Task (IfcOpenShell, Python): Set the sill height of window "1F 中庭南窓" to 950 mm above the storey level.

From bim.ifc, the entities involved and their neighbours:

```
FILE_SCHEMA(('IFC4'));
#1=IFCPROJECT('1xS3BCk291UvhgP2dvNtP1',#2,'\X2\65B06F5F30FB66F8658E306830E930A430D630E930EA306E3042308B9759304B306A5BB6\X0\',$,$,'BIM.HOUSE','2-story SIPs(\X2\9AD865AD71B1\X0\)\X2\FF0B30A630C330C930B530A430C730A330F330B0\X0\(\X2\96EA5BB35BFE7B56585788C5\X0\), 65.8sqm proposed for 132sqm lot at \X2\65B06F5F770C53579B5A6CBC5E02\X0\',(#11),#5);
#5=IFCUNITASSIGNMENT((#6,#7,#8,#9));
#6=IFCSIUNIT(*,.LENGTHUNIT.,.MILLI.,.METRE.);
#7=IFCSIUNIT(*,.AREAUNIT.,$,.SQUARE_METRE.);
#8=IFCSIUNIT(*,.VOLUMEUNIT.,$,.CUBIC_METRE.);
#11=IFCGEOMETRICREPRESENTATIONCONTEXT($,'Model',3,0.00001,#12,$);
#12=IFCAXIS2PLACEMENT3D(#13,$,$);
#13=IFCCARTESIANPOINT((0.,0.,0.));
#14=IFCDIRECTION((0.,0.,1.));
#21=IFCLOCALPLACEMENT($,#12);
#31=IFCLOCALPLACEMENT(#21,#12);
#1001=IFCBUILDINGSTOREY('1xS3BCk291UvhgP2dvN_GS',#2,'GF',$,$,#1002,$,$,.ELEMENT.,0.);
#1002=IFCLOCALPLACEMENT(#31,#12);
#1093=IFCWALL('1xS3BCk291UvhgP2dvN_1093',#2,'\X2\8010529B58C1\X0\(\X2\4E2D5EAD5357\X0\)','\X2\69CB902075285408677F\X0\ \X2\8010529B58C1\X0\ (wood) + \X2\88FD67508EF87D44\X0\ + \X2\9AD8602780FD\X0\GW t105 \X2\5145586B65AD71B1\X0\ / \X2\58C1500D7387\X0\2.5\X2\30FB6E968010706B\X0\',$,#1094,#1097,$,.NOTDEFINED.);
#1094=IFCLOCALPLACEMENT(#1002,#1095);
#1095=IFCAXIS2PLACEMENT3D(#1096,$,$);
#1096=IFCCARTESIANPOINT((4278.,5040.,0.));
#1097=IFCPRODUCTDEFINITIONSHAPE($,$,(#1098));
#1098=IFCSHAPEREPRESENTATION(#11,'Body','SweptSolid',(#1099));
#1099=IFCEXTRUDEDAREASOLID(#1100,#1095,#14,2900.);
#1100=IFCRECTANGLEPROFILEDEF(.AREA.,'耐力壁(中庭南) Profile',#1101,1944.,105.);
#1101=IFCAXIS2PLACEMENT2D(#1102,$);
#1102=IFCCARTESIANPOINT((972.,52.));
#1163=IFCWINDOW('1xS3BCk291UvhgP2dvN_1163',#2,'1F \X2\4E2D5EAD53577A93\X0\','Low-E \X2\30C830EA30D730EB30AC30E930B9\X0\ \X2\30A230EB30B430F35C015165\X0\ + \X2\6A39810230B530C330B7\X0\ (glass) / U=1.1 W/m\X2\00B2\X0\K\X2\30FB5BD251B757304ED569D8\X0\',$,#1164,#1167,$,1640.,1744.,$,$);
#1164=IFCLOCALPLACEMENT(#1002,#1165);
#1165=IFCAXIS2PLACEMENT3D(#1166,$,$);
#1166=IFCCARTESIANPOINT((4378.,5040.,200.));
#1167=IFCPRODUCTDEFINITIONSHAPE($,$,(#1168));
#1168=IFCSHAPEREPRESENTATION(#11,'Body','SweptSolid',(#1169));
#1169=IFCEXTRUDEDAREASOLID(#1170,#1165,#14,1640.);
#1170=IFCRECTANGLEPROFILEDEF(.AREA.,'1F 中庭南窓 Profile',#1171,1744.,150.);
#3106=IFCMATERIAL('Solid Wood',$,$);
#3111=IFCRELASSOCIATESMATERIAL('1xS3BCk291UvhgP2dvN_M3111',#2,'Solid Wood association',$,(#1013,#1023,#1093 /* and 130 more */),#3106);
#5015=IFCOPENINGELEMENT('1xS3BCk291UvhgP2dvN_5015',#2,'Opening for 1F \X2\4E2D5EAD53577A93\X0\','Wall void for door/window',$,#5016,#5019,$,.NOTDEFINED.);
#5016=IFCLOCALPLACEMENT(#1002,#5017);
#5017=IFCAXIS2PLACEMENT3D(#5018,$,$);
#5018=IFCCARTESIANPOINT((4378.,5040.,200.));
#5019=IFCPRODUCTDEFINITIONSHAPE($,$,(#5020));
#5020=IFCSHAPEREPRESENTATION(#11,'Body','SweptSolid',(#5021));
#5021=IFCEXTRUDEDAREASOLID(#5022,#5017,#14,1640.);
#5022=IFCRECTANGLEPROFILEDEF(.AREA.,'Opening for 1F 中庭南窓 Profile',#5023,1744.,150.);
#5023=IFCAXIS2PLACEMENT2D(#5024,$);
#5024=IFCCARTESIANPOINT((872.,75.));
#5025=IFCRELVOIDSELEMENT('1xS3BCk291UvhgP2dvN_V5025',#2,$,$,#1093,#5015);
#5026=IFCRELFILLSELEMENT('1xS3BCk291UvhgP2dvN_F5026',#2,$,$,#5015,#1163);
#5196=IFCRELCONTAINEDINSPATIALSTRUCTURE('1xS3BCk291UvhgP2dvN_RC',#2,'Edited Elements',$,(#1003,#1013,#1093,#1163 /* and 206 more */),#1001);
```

```python
import numpy as np
import ifcopenshell
import ifcopenshell.api.geometry
import ifcopenshell.geom
import ifcopenshell.util.element
import ifcopenshell.util.placement
import ifcopenshell.util.shape
import ifcopenshell.util.unit

model = ifcopenshell.open("bim.ifc")
unit_scale = ifcopenshell.util.unit.calculate_unit_scale(model)

window = model.by_guid("1xS3BCk291UvhgP2dvN_1163")
opening = window.FillsVoids[0].RelatingOpeningElement
storey = ifcopenshell.util.element.get_container(window, ifc_class="IfcBuildingStorey")
level = ifcopenshell.util.placement.get_local_placement(storey.ObjectPlacement)[2, 3]

# The opening's origin need not be at the sill, so measure its lowest point.
shape = ifcopenshell.geom.create_shape(ifcopenshell.geom.settings(), opening)
bottom = ifcopenshell.util.shape.get_shape_bottom_elevation(shape, shape.geometry) / unit_scale
dz = level + 950.0 - bottom

shift = np.array([0.0, 0.0, dz])
# The window is not placed relative to its opening, so move both.
for product in (opening, window):
    matrix = ifcopenshell.util.placement.get_local_placement(product.ObjectPlacement)
    matrix[:3, 3] += shift
    ifcopenshell.api.geometry.edit_object_placement(model, product=product, matrix=matrix, is_si=False)

print(f"moved by {dz * unit_scale:+.3f} m")

model.write("bim_updated.ifc")
```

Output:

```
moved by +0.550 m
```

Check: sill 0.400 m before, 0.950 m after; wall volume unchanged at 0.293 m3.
